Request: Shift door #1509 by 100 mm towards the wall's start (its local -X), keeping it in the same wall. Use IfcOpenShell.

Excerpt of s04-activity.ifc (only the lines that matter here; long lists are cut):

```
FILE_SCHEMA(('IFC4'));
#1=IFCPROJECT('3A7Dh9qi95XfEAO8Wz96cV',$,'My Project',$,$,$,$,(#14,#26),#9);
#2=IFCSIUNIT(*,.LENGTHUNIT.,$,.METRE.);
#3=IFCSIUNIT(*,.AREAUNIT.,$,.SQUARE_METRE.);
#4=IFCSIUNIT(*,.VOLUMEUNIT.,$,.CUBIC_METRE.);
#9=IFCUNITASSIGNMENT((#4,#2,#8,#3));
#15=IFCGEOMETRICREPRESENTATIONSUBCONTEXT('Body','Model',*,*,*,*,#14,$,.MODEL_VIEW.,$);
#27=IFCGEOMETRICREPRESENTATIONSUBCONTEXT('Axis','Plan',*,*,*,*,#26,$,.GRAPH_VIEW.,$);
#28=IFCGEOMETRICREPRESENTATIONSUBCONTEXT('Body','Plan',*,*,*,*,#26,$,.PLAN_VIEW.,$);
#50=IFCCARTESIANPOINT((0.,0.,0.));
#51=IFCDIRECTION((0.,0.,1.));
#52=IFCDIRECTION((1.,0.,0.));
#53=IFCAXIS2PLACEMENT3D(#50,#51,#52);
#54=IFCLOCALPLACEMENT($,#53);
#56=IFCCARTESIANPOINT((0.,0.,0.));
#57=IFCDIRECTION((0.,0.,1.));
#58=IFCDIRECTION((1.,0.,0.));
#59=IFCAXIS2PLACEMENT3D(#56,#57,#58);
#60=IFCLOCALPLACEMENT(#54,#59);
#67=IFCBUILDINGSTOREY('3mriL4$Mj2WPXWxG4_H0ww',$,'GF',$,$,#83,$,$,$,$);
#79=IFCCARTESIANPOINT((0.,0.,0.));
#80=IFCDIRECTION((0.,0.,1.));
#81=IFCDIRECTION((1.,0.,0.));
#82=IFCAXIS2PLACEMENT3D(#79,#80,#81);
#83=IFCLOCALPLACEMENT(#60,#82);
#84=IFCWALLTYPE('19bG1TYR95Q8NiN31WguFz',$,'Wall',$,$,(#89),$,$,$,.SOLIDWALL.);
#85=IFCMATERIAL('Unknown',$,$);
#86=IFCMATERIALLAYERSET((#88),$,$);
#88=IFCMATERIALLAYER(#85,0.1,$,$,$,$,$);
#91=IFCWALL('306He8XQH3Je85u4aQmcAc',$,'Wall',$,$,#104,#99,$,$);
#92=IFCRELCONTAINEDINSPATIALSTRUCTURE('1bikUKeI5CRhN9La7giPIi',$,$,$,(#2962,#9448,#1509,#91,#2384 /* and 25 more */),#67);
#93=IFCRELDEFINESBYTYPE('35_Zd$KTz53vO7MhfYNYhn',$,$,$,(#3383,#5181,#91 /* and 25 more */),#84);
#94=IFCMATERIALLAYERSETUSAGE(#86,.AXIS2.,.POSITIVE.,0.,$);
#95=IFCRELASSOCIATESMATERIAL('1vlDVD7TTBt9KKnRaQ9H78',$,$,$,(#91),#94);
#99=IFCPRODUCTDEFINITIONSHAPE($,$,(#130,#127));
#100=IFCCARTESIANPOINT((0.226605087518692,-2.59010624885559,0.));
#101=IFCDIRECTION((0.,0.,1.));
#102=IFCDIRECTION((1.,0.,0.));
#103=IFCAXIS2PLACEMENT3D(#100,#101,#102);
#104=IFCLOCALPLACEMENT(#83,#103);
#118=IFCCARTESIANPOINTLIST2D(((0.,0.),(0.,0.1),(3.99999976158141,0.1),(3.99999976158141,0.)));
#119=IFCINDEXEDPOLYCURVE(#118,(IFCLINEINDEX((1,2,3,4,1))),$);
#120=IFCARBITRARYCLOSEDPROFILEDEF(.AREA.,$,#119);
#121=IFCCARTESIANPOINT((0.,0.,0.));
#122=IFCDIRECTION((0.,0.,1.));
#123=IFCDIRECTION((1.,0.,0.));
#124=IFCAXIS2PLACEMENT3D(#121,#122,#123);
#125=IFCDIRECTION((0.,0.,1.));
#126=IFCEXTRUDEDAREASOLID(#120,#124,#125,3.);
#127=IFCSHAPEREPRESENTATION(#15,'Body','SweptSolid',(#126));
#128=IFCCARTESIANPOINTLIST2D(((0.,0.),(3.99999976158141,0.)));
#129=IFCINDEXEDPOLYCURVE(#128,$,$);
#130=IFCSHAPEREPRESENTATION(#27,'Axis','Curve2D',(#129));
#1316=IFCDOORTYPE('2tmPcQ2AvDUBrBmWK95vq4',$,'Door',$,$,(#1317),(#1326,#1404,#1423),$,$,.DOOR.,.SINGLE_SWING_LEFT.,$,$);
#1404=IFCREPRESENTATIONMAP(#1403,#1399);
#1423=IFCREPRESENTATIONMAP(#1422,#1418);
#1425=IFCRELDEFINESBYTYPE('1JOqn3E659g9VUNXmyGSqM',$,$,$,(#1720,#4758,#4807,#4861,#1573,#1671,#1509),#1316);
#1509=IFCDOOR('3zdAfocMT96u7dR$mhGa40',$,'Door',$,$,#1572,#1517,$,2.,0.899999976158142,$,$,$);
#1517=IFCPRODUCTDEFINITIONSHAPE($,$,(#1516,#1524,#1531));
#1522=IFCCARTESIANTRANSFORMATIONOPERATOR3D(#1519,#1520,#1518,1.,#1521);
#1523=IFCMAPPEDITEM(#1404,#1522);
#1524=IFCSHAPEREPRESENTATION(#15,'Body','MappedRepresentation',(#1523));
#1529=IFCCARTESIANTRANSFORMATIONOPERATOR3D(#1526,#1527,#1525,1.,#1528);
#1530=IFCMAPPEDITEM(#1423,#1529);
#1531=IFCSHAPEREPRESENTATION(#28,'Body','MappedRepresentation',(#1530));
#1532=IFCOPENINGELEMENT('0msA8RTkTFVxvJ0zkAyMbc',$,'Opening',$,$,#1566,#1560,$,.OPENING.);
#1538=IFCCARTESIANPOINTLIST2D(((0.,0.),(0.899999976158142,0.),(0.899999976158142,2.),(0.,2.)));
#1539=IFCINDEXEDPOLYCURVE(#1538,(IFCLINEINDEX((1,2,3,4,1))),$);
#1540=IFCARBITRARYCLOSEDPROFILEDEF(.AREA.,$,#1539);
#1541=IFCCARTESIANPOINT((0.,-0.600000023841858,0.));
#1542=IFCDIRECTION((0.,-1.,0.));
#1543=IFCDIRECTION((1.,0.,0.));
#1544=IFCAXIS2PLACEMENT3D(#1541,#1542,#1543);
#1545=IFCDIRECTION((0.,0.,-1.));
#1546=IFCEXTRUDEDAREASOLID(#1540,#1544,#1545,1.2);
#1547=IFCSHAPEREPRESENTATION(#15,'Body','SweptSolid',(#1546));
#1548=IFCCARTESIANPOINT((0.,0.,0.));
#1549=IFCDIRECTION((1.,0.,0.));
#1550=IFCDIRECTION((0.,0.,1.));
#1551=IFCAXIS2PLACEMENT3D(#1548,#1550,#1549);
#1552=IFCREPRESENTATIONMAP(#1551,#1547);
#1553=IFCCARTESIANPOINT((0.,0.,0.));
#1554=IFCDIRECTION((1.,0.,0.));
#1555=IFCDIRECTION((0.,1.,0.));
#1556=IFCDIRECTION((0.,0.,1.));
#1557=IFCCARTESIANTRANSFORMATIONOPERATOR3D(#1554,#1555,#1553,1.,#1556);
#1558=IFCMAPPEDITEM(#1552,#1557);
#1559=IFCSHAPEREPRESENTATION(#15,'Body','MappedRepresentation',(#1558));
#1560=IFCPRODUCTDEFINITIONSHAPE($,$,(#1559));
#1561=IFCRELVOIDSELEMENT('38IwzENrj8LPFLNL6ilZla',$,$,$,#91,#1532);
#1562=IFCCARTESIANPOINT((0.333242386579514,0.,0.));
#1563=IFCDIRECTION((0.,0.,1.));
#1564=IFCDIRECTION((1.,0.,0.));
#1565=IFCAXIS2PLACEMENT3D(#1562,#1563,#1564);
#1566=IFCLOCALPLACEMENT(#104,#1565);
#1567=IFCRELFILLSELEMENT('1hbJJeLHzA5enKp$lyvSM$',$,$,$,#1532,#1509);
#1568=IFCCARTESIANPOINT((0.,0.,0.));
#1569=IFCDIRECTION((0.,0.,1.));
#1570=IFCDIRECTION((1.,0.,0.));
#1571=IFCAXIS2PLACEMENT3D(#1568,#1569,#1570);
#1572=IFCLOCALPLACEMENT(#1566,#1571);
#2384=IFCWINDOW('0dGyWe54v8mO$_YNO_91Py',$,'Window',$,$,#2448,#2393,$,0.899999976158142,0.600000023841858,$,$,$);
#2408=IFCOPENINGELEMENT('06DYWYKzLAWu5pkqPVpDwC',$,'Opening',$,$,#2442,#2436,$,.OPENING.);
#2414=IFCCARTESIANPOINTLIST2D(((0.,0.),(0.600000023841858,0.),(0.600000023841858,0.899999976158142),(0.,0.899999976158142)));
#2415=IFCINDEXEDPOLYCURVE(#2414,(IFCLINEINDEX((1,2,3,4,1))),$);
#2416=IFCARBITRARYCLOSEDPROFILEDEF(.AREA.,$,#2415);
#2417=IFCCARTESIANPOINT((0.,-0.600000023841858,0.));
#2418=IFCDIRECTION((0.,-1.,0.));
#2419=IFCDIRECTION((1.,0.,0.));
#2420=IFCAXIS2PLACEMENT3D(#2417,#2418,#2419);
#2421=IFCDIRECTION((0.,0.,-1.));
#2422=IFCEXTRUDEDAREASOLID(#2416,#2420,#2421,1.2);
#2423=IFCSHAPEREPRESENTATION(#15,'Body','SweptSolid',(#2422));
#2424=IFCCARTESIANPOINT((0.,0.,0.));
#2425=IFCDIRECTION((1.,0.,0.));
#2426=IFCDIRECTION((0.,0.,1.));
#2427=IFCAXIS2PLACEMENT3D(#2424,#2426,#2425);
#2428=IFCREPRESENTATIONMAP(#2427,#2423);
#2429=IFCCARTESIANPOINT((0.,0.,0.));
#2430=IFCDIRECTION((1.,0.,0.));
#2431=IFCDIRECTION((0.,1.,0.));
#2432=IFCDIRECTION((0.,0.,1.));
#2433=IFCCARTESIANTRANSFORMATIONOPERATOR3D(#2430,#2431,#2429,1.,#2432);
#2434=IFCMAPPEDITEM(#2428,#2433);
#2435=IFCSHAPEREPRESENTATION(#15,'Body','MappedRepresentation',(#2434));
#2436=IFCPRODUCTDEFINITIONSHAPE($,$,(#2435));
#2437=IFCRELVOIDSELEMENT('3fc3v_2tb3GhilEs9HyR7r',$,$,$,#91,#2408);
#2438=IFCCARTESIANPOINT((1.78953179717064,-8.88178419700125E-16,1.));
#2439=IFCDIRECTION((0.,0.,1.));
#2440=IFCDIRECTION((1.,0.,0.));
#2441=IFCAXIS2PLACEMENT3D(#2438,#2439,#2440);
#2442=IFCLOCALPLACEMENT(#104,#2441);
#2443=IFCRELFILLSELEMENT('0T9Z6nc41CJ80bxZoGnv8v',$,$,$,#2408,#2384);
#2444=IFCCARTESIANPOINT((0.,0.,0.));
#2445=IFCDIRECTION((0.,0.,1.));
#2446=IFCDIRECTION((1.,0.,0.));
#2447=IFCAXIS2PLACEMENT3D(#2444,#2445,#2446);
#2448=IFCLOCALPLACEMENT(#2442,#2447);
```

```python
import ifcopenshell
import ifcopenshell.api.geometry
import ifcopenshell.util.placement
import ifcopenshell.util.unit

model = ifcopenshell.open("s04-activity.ifc")
unit_scale = ifcopenshell.util.unit.calculate_unit_scale(model)

door = model.by_guid("3zdAfocMT96u7dR$mhGa40")
opening = door.FillsVoids[0].RelatingOpeningElement
wall = opening.VoidsElements[0].RelatingBuildingElement

wall_matrix = ifcopenshell.util.placement.get_local_placement(wall.ObjectPlacement)
shift = wall_matrix[:3, 0] * -0.1 / unit_scale
before = ifcopenshell.util.placement.get_local_placement(door.ObjectPlacement)[:3, 3].copy()

# The door is placed relative to its opening, so it follows when the opening moves.
matrix = ifcopenshell.util.placement.get_local_placement(opening.ObjectPlacement)
matrix[:3, 3] += shift
ifcopenshell.api.geometry.edit_object_placement(
    model, product=opening, matrix=matrix, is_si=False, should_transform_children=True
)

after = ifcopenshell.util.placement.get_local_placement(door.ObjectPlacement)[:3, 3]
print("door moved by", (after - before).round(3) + 0.0)

model.write("s04-activity_rev.ifc")
```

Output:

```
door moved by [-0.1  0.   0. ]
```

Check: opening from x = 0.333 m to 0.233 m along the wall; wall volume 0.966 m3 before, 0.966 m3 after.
